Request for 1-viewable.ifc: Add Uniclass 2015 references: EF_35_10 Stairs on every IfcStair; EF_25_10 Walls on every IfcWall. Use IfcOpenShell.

First a look at what the model holds.

```python
import ifcopenshell

model = ifcopenshell.open("1-viewable.ifc")
print(model.schema)
print("classifications:", [c.Name for c in model.by_type("IfcClassification")])
for ifc_class in ("IfcDoor", "IfcRoof", "IfcStair", "IfcWall", "IfcWindow"):
    print(ifc_class, len(model.by_type(ifc_class)))
```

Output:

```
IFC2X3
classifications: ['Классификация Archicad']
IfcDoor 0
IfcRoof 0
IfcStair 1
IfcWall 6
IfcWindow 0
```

```python
import ifcopenshell
import ifcopenshell.api.classification

model = ifcopenshell.open("1-viewable.ifc")

# IFC2X3 requires Source and Edition and has no link from the project to the system.
system = model.create_entity("IfcClassification", Source="NBS", Edition="2015", Name="Uniclass 2015")

codes = {
    "IfcStair": ("EF_35_10", "Stairs"),
    "IfcWall": ("EF_25_10", "Walls"),
}
for ifc_class, (code, name) in codes.items():
    products = model.by_type(ifc_class)
    ifcopenshell.api.classification.add_reference(
        model, products=products, classification=system, identification=code, name=name
    )
    print(code, len(products))

model.write("1-viewable_v2.ifc")
```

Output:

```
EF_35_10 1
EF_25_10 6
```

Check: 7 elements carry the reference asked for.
